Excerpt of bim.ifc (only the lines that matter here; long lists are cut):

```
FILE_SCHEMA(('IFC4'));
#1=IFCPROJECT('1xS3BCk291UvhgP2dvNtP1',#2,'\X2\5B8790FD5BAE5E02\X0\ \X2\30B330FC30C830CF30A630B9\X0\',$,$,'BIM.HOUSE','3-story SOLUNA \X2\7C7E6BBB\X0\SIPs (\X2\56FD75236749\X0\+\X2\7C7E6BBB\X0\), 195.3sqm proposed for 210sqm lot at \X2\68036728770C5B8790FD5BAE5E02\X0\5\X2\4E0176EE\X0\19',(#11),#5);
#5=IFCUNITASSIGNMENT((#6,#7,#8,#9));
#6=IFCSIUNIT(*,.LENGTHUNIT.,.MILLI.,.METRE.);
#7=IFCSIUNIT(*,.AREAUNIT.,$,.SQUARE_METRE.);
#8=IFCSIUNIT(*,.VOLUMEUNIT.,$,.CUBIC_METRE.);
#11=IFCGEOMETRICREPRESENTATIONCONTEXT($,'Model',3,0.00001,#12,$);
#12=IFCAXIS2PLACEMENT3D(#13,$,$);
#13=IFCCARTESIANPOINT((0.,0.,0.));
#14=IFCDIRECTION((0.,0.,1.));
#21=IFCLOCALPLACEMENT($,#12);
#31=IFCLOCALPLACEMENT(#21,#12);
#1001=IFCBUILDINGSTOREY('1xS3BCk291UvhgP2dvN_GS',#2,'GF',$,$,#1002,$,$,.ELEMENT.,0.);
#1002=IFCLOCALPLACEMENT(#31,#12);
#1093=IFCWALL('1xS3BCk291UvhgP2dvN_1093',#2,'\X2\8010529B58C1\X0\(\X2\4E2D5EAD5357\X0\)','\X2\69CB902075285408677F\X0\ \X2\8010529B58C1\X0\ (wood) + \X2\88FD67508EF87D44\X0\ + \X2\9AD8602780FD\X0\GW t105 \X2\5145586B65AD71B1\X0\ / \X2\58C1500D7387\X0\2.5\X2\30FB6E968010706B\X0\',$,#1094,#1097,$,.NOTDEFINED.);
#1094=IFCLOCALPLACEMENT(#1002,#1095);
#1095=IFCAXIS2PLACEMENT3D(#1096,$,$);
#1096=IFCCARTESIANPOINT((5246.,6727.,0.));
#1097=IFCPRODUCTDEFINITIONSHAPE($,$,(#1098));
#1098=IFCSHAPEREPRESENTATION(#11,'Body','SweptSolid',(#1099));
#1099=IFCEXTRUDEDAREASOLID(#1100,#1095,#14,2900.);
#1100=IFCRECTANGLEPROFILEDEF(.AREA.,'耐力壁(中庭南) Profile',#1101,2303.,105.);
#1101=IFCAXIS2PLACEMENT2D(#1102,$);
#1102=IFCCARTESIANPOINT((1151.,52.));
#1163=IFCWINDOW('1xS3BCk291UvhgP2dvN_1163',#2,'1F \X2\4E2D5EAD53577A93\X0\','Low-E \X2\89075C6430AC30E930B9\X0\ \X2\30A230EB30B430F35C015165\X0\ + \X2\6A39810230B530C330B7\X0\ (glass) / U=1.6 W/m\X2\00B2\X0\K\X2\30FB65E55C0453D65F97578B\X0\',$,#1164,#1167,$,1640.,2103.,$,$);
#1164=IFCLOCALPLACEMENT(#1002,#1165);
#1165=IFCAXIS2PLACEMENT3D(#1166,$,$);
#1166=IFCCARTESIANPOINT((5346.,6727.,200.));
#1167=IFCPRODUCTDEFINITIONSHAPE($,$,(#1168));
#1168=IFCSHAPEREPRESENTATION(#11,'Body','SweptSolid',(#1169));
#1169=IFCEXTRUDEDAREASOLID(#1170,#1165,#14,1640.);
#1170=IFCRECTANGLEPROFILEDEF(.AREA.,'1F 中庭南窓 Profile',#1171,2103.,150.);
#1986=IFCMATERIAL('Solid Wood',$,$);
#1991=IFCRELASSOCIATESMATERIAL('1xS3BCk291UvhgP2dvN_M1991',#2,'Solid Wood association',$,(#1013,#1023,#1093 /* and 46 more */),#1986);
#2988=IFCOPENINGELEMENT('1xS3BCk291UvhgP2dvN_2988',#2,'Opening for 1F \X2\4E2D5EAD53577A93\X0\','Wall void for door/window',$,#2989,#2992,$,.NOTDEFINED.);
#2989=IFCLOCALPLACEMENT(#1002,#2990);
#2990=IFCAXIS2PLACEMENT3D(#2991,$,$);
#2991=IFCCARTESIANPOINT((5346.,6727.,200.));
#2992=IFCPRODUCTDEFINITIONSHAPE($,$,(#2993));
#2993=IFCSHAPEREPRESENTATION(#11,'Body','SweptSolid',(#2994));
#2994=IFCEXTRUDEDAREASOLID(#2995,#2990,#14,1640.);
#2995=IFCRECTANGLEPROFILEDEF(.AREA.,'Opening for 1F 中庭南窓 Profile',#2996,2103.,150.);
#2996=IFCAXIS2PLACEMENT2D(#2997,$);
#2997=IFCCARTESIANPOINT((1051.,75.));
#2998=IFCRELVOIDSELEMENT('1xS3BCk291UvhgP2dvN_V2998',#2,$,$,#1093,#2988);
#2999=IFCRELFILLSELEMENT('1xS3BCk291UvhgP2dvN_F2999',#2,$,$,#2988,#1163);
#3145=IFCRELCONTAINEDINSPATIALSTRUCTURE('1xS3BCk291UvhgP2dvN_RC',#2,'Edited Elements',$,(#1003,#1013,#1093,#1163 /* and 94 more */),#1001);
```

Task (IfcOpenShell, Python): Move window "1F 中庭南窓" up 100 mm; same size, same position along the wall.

```python
import numpy as np
import ifcopenshell
import ifcopenshell.api.geometry
import ifcopenshell.util.placement
import ifcopenshell.util.unit

model = ifcopenshell.open("bim.ifc")
unit_scale = ifcopenshell.util.unit.calculate_unit_scale(model)

window = model.by_guid("1xS3BCk291UvhgP2dvN_1163")
opening = window.FillsVoids[0].RelatingOpeningElement
dz = 0.1 / unit_scale

shift = np.array([0.0, 0.0, dz])
# The window is not placed relative to its opening, so move both.
for product in (opening, window):
    matrix = ifcopenshell.util.placement.get_local_placement(product.ObjectPlacement)
    matrix[:3, 3] += shift
    ifcopenshell.api.geometry.edit_object_placement(model, product=product, matrix=matrix, is_si=False)

print(f"moved by {dz * unit_scale:+.3f} m")

model.write("bim_v2.ifc")
```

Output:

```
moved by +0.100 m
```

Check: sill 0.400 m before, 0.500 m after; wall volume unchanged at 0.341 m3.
